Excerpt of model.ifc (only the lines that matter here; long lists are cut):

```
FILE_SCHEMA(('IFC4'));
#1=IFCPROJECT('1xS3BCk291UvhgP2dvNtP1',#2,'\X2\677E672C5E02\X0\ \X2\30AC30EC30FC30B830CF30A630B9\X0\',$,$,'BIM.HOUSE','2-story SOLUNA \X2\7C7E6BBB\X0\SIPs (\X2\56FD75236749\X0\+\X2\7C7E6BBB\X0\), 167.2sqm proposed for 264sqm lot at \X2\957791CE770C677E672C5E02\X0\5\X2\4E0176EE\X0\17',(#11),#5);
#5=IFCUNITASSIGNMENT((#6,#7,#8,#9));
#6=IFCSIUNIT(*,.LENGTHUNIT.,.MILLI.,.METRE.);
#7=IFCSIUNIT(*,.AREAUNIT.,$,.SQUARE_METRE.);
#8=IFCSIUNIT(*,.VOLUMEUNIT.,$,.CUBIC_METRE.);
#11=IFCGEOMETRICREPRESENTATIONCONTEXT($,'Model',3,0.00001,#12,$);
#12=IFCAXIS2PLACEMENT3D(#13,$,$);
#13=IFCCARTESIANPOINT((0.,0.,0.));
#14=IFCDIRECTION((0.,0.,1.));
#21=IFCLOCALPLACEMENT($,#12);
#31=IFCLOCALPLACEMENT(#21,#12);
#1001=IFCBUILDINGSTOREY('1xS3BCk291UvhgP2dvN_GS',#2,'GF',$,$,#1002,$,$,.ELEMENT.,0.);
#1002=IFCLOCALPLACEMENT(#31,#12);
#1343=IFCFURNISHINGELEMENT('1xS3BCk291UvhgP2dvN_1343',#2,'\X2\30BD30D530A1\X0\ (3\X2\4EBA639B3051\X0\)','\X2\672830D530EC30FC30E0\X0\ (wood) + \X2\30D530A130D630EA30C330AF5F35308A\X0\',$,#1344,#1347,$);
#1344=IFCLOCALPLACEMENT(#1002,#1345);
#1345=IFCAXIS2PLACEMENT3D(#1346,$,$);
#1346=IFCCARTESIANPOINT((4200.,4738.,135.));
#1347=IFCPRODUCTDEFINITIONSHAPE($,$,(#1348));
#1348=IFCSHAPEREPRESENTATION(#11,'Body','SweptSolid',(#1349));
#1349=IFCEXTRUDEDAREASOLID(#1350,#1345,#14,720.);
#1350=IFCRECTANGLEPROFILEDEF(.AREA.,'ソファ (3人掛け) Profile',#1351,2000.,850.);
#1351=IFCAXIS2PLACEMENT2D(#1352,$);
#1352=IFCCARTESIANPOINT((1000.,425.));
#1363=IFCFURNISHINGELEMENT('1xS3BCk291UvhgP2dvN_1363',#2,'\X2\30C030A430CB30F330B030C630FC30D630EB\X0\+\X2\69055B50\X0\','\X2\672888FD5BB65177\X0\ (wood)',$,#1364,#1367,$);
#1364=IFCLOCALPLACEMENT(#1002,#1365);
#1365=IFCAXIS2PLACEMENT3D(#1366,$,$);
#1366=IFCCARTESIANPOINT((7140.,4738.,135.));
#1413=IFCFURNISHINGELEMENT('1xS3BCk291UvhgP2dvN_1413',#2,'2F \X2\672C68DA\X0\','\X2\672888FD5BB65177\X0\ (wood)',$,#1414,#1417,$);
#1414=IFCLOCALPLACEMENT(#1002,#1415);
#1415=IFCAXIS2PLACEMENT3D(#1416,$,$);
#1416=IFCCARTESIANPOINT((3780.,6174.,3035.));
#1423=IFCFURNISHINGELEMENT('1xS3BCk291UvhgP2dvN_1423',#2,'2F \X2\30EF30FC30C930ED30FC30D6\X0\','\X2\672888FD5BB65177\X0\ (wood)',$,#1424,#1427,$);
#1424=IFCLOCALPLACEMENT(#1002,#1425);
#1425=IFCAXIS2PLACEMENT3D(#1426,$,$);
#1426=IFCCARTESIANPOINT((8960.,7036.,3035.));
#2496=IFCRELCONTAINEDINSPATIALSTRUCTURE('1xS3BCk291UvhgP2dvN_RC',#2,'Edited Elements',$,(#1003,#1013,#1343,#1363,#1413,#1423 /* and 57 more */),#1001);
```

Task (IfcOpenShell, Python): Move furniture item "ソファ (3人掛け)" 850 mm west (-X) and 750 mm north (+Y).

```python
import ifcopenshell
import ifcopenshell.api.geometry
import ifcopenshell.util.placement
import ifcopenshell.util.unit

model = ifcopenshell.open("model.ifc")
unit_scale = ifcopenshell.util.unit.calculate_unit_scale(model)

item = model.by_guid("1xS3BCk291UvhgP2dvN_1343")
matrix = ifcopenshell.util.placement.get_local_placement(item.ObjectPlacement)
matrix[0, 3] -= 0.85 / unit_scale
matrix[1, 3] += 0.75 / unit_scale
ifcopenshell.api.geometry.edit_object_placement(model, product=item, matrix=matrix, is_si=False)

print(ifcopenshell.util.placement.get_local_placement(item.ObjectPlacement).round(3) + 0.0)

model.write("model_v2.ifc")
```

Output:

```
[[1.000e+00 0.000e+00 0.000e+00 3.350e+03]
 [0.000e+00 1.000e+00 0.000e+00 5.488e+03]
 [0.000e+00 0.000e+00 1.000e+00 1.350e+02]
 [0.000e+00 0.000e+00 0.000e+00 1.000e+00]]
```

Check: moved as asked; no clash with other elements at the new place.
